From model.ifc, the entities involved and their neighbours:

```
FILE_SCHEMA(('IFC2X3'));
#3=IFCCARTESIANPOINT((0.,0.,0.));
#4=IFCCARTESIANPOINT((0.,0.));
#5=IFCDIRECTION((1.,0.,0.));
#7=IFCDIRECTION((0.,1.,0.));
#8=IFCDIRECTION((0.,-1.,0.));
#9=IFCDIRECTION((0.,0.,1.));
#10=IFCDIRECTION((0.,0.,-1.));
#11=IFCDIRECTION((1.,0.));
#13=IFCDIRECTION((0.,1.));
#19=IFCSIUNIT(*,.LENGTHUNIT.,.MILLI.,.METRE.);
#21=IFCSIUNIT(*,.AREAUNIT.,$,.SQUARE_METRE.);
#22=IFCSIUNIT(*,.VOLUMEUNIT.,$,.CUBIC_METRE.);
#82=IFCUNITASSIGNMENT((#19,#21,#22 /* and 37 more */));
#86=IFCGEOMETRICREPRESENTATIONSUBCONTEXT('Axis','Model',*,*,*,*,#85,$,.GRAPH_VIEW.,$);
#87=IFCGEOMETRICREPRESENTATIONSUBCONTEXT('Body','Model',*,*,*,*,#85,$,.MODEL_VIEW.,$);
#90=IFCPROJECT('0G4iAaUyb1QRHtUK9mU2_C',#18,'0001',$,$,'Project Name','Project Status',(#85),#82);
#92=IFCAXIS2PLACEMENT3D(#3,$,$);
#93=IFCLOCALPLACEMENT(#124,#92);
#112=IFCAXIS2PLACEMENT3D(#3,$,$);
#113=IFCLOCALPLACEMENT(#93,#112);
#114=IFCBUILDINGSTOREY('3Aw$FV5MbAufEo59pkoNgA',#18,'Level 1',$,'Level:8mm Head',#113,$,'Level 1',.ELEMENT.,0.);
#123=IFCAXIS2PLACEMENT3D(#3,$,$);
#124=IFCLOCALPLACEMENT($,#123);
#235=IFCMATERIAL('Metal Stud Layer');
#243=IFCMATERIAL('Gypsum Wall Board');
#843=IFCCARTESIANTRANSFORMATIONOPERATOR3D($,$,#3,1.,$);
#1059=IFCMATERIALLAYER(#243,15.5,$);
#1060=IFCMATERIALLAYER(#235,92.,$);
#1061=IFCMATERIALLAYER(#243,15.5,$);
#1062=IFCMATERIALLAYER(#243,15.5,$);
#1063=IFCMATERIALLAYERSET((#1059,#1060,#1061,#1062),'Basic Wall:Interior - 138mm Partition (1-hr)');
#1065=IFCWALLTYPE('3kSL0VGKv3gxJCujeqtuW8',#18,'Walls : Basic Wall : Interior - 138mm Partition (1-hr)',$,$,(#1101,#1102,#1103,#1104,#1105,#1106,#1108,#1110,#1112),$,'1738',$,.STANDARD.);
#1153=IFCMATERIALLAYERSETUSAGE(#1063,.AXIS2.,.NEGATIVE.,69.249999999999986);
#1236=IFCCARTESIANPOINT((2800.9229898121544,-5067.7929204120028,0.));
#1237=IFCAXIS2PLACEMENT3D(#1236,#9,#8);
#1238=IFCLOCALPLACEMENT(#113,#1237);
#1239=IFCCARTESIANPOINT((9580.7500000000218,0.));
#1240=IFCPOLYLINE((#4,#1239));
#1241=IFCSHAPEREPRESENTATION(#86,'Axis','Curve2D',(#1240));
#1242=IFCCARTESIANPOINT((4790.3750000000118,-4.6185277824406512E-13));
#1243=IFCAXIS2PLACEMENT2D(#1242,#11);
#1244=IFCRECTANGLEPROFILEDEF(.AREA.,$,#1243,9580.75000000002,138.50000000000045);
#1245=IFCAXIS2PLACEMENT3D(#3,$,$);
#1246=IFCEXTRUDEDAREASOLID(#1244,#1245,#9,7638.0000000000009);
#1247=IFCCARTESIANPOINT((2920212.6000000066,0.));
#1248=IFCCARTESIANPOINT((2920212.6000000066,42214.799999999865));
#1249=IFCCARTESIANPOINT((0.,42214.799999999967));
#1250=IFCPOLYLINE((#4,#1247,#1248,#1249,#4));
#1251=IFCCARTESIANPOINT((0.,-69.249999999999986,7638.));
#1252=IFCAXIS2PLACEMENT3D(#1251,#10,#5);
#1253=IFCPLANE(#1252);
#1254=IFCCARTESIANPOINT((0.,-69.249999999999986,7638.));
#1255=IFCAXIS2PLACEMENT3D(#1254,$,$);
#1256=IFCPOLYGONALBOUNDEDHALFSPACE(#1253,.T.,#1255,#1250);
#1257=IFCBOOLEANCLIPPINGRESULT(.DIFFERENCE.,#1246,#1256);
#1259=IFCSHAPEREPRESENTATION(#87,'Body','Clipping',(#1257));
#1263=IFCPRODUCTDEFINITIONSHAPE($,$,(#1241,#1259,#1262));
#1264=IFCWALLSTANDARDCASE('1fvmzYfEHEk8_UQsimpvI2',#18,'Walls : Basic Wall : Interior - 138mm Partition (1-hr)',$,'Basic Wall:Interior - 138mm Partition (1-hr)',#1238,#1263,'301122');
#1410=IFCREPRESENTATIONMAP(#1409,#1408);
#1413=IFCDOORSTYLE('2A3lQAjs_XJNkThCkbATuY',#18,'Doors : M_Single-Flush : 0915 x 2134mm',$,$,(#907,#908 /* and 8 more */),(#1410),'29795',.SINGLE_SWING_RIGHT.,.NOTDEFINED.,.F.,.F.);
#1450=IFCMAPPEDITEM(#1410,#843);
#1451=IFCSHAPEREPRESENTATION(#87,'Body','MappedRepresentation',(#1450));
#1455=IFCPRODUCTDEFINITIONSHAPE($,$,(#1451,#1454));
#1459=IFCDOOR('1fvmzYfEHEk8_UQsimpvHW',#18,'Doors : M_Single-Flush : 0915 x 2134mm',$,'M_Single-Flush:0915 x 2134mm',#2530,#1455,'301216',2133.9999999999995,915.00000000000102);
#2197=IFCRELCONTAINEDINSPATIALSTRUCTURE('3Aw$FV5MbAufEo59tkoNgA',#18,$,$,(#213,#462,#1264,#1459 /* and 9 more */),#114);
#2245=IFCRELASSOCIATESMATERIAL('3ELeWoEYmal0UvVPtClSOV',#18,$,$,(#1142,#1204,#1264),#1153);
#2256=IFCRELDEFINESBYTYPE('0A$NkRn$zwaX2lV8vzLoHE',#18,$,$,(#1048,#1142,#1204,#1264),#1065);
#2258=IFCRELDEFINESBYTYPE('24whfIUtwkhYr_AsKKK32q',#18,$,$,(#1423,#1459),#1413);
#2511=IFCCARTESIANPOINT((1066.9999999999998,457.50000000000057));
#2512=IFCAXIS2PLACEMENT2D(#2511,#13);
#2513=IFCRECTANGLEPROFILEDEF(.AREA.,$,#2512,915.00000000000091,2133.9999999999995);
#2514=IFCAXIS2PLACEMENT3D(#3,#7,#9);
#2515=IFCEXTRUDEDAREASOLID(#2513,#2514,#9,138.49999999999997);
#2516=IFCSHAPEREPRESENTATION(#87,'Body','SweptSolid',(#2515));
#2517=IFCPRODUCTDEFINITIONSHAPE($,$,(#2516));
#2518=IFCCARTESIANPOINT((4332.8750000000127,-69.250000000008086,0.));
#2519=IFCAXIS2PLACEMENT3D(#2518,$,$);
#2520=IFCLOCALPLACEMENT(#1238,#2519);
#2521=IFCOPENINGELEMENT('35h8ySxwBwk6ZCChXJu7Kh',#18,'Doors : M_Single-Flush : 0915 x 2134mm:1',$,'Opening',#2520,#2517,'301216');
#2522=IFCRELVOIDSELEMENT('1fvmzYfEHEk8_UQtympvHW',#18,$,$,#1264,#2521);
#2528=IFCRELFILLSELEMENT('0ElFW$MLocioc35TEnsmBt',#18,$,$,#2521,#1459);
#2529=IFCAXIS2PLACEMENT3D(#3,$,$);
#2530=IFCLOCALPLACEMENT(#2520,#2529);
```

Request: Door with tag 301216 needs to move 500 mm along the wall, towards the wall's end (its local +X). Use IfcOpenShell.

```python
import ifcopenshell
import ifcopenshell.api.geometry
import ifcopenshell.util.placement
import ifcopenshell.util.unit

model = ifcopenshell.open("model.ifc")
unit_scale = ifcopenshell.util.unit.calculate_unit_scale(model)

door = model.by_guid("1fvmzYfEHEk8_UQsimpvHW")
opening = door.FillsVoids[0].RelatingOpeningElement
wall = opening.VoidsElements[0].RelatingBuildingElement

wall_matrix = ifcopenshell.util.placement.get_local_placement(wall.ObjectPlacement)
shift = wall_matrix[:3, 0] * 0.5 / unit_scale
before = ifcopenshell.util.placement.get_local_placement(door.ObjectPlacement)[:3, 3].copy()

# The door is placed relative to its opening, so it follows when the opening moves.
matrix = ifcopenshell.util.placement.get_local_placement(opening.ObjectPlacement)
matrix[:3, 3] += shift
ifcopenshell.api.geometry.edit_object_placement(
    model, product=opening, matrix=matrix, is_si=False, should_transform_children=True
)

after = ifcopenshell.util.placement.get_local_placement(door.ObjectPlacement)[:3, 3]
print("door moved by", (after - before).round(3) + 0.0)

model.write("model-out.ifc")
```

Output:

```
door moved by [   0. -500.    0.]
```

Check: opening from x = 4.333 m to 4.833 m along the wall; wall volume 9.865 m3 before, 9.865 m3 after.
